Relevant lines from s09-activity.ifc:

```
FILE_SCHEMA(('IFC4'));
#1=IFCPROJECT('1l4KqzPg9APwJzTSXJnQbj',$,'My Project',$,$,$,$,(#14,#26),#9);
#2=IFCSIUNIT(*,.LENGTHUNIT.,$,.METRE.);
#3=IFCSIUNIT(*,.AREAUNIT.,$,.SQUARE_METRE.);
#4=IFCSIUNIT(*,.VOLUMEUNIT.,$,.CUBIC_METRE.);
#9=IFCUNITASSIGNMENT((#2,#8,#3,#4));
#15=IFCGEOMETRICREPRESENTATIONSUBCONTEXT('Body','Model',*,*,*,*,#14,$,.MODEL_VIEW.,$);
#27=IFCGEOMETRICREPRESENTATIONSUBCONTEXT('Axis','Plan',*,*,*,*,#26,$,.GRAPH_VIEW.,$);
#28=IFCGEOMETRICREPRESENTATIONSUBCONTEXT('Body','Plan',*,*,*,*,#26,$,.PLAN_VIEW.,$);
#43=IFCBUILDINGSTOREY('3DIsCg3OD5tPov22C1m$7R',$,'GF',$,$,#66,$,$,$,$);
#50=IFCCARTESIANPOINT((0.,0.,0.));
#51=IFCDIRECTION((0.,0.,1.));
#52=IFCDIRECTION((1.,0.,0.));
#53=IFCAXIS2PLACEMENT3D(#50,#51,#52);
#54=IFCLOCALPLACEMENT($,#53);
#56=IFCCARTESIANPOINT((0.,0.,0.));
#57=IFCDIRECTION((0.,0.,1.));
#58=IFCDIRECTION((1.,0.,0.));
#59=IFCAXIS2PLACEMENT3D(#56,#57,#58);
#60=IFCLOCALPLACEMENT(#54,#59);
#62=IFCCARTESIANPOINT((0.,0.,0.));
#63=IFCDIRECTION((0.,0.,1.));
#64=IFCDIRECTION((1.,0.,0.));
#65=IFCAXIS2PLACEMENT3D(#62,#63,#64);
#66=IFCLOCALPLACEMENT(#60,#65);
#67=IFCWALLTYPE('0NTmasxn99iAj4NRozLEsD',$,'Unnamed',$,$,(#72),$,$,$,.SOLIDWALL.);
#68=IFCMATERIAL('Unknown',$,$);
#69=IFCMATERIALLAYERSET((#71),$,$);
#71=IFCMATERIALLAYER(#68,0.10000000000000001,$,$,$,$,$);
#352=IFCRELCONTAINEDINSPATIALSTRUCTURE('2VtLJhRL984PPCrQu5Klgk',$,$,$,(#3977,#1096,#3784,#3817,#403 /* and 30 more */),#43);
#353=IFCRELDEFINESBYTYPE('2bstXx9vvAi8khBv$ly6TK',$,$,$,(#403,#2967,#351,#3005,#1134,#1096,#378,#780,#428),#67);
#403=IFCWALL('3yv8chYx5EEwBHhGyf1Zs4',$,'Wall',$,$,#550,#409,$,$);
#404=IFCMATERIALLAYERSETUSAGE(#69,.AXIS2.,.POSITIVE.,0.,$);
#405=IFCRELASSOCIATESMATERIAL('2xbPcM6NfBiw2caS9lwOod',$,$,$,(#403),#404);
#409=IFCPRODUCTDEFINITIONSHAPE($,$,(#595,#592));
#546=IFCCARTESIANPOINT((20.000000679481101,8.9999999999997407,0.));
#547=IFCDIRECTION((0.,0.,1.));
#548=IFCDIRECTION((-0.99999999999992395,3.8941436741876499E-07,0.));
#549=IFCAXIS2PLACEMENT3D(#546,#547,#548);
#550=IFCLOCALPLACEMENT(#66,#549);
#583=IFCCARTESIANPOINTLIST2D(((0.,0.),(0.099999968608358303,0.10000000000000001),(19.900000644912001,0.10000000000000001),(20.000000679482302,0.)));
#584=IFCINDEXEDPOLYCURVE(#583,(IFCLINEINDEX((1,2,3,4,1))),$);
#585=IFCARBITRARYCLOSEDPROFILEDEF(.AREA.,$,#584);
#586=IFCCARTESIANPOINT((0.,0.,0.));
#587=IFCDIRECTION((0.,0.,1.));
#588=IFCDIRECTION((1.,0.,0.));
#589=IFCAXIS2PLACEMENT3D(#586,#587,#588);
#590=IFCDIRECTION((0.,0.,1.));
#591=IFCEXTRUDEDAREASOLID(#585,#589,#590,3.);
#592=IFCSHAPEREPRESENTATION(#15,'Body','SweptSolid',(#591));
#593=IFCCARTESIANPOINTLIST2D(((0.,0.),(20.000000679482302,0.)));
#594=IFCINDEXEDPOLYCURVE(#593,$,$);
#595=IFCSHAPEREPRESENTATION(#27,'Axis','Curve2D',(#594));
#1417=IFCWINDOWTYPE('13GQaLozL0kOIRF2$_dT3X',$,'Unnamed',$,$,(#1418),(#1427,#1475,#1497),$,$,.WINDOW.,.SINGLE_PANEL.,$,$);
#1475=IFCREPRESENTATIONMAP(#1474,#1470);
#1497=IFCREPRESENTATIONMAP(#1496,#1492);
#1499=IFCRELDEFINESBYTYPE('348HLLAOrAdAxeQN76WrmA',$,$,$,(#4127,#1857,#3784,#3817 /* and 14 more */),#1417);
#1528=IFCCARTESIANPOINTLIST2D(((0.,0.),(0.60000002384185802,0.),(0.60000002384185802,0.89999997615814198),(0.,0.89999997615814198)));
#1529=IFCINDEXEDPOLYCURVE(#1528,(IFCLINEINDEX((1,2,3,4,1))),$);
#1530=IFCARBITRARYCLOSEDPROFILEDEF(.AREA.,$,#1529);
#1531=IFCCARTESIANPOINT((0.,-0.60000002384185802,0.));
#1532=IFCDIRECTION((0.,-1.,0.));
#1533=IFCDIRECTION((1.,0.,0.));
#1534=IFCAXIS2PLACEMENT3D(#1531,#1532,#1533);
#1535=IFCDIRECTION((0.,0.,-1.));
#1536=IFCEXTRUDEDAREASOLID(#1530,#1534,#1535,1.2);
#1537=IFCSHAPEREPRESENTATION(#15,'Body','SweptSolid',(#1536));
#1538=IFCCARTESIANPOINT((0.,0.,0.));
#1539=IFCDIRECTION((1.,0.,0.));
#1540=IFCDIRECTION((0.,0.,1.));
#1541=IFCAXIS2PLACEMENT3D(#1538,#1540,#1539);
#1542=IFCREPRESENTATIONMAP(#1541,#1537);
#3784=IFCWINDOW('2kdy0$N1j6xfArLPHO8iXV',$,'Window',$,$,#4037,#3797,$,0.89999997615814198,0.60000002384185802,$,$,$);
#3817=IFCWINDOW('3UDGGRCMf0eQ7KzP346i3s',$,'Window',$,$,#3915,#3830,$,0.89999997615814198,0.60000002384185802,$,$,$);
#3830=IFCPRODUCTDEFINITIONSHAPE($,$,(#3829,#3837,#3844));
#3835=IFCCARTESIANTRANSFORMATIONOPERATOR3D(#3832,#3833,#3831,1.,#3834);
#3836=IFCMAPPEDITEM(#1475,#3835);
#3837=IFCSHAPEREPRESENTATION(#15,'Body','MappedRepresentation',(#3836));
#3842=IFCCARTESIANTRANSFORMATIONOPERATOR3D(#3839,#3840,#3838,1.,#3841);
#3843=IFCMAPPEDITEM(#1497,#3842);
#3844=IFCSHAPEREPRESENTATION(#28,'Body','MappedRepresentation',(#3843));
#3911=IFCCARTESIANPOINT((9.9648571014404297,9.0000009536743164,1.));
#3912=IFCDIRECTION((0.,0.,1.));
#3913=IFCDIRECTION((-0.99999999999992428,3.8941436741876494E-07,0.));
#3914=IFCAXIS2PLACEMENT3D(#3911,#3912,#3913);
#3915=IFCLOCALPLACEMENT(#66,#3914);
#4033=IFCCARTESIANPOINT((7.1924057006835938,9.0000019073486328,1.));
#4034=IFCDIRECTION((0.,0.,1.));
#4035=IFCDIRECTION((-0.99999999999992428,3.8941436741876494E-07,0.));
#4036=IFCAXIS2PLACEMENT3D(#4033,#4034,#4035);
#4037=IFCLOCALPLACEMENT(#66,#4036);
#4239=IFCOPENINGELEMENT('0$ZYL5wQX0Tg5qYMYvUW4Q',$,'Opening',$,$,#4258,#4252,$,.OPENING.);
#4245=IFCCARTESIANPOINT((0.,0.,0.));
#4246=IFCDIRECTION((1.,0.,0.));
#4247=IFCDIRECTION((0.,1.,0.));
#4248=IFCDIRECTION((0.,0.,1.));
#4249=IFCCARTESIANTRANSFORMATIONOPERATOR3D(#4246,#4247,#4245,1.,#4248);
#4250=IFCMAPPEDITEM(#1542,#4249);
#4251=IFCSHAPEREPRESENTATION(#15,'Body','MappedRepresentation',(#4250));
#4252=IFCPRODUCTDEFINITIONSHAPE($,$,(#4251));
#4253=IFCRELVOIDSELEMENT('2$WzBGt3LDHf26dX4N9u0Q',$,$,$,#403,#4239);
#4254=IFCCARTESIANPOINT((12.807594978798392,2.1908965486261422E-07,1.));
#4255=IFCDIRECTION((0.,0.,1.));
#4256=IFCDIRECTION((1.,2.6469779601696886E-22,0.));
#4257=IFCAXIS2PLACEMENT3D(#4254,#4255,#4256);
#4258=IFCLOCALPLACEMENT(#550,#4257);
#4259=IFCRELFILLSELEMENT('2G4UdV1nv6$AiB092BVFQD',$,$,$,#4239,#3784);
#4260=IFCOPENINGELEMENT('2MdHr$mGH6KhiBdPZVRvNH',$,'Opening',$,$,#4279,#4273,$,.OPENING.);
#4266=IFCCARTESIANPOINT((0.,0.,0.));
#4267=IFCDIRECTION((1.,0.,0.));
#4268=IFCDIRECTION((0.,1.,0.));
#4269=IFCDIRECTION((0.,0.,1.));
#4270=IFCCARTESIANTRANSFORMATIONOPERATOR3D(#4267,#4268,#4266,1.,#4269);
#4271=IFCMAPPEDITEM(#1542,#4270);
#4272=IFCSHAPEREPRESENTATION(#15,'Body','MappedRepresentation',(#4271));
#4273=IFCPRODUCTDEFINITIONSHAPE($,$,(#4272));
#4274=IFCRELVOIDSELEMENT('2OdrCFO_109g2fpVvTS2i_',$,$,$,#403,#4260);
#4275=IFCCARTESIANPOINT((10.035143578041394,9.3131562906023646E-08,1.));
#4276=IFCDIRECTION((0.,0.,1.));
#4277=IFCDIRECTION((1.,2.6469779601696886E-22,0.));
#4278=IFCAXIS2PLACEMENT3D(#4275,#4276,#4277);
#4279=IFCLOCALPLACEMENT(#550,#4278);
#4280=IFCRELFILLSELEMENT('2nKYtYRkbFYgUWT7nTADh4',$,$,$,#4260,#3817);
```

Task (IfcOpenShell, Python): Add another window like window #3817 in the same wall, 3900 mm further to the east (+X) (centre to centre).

```python
import ifcopenshell
import ifcopenshell.api.feature
import ifcopenshell.api.geometry
import ifcopenshell.api.root
import ifcopenshell.geom
import ifcopenshell.util.element
import ifcopenshell.util.placement
import ifcopenshell.util.shape
import ifcopenshell.util.unit

model = ifcopenshell.open("s09-activity.ifc")
unit_scale = ifcopenshell.util.unit.calculate_unit_scale(model)
settings = ifcopenshell.geom.settings()


def volume(element):
    """Net volume in cubic metres, openings subtracted."""
    shape = ifcopenshell.geom.create_shape(settings, element)
    return ifcopenshell.util.shape.get_volume(shape.geometry)


window = model.by_guid("3UDGGRCMf0eQ7KzP346i3s")
opening = window.FillsVoids[0].RelatingOpeningElement
wall = opening.VoidsElements[0].RelatingBuildingElement
before = volume(wall)
shift = ifcopenshell.util.placement.get_local_placement(wall.ObjectPlacement)[:3, 0] * -3.9 / unit_scale

# copy_class copies the void relationship, type, container and properties, but no geometry.
new_opening = ifcopenshell.api.root.copy_class(model, product=opening)
new_opening.Representation = ifcopenshell.util.element.copy_deep(
    model, opening.Representation, exclude=["IfcGeometricRepresentationContext", "IfcRepresentationMap"]
)
new_window = ifcopenshell.api.root.copy_class(model, product=window)
new_window.Representation = ifcopenshell.util.element.copy_deep(
    model, window.Representation, exclude=["IfcGeometricRepresentationContext", "IfcRepresentationMap"]
)
ifcopenshell.api.feature.add_filling(model, opening=new_opening, element=new_window)

for old, new in ((opening, new_opening), (window, new_window)):
    matrix = ifcopenshell.util.placement.get_local_placement(old.ObjectPlacement)
    matrix[:3, 3] += shift
    ifcopenshell.api.geometry.edit_object_placement(model, product=new, matrix=matrix, is_si=False)

after = volume(wall)

print(f"wall volume {before:.3f} -> {after:.3f} m3")

model.write("s09-activity_edited.ifc")
```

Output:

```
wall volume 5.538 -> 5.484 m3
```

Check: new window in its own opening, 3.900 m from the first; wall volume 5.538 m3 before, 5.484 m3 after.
